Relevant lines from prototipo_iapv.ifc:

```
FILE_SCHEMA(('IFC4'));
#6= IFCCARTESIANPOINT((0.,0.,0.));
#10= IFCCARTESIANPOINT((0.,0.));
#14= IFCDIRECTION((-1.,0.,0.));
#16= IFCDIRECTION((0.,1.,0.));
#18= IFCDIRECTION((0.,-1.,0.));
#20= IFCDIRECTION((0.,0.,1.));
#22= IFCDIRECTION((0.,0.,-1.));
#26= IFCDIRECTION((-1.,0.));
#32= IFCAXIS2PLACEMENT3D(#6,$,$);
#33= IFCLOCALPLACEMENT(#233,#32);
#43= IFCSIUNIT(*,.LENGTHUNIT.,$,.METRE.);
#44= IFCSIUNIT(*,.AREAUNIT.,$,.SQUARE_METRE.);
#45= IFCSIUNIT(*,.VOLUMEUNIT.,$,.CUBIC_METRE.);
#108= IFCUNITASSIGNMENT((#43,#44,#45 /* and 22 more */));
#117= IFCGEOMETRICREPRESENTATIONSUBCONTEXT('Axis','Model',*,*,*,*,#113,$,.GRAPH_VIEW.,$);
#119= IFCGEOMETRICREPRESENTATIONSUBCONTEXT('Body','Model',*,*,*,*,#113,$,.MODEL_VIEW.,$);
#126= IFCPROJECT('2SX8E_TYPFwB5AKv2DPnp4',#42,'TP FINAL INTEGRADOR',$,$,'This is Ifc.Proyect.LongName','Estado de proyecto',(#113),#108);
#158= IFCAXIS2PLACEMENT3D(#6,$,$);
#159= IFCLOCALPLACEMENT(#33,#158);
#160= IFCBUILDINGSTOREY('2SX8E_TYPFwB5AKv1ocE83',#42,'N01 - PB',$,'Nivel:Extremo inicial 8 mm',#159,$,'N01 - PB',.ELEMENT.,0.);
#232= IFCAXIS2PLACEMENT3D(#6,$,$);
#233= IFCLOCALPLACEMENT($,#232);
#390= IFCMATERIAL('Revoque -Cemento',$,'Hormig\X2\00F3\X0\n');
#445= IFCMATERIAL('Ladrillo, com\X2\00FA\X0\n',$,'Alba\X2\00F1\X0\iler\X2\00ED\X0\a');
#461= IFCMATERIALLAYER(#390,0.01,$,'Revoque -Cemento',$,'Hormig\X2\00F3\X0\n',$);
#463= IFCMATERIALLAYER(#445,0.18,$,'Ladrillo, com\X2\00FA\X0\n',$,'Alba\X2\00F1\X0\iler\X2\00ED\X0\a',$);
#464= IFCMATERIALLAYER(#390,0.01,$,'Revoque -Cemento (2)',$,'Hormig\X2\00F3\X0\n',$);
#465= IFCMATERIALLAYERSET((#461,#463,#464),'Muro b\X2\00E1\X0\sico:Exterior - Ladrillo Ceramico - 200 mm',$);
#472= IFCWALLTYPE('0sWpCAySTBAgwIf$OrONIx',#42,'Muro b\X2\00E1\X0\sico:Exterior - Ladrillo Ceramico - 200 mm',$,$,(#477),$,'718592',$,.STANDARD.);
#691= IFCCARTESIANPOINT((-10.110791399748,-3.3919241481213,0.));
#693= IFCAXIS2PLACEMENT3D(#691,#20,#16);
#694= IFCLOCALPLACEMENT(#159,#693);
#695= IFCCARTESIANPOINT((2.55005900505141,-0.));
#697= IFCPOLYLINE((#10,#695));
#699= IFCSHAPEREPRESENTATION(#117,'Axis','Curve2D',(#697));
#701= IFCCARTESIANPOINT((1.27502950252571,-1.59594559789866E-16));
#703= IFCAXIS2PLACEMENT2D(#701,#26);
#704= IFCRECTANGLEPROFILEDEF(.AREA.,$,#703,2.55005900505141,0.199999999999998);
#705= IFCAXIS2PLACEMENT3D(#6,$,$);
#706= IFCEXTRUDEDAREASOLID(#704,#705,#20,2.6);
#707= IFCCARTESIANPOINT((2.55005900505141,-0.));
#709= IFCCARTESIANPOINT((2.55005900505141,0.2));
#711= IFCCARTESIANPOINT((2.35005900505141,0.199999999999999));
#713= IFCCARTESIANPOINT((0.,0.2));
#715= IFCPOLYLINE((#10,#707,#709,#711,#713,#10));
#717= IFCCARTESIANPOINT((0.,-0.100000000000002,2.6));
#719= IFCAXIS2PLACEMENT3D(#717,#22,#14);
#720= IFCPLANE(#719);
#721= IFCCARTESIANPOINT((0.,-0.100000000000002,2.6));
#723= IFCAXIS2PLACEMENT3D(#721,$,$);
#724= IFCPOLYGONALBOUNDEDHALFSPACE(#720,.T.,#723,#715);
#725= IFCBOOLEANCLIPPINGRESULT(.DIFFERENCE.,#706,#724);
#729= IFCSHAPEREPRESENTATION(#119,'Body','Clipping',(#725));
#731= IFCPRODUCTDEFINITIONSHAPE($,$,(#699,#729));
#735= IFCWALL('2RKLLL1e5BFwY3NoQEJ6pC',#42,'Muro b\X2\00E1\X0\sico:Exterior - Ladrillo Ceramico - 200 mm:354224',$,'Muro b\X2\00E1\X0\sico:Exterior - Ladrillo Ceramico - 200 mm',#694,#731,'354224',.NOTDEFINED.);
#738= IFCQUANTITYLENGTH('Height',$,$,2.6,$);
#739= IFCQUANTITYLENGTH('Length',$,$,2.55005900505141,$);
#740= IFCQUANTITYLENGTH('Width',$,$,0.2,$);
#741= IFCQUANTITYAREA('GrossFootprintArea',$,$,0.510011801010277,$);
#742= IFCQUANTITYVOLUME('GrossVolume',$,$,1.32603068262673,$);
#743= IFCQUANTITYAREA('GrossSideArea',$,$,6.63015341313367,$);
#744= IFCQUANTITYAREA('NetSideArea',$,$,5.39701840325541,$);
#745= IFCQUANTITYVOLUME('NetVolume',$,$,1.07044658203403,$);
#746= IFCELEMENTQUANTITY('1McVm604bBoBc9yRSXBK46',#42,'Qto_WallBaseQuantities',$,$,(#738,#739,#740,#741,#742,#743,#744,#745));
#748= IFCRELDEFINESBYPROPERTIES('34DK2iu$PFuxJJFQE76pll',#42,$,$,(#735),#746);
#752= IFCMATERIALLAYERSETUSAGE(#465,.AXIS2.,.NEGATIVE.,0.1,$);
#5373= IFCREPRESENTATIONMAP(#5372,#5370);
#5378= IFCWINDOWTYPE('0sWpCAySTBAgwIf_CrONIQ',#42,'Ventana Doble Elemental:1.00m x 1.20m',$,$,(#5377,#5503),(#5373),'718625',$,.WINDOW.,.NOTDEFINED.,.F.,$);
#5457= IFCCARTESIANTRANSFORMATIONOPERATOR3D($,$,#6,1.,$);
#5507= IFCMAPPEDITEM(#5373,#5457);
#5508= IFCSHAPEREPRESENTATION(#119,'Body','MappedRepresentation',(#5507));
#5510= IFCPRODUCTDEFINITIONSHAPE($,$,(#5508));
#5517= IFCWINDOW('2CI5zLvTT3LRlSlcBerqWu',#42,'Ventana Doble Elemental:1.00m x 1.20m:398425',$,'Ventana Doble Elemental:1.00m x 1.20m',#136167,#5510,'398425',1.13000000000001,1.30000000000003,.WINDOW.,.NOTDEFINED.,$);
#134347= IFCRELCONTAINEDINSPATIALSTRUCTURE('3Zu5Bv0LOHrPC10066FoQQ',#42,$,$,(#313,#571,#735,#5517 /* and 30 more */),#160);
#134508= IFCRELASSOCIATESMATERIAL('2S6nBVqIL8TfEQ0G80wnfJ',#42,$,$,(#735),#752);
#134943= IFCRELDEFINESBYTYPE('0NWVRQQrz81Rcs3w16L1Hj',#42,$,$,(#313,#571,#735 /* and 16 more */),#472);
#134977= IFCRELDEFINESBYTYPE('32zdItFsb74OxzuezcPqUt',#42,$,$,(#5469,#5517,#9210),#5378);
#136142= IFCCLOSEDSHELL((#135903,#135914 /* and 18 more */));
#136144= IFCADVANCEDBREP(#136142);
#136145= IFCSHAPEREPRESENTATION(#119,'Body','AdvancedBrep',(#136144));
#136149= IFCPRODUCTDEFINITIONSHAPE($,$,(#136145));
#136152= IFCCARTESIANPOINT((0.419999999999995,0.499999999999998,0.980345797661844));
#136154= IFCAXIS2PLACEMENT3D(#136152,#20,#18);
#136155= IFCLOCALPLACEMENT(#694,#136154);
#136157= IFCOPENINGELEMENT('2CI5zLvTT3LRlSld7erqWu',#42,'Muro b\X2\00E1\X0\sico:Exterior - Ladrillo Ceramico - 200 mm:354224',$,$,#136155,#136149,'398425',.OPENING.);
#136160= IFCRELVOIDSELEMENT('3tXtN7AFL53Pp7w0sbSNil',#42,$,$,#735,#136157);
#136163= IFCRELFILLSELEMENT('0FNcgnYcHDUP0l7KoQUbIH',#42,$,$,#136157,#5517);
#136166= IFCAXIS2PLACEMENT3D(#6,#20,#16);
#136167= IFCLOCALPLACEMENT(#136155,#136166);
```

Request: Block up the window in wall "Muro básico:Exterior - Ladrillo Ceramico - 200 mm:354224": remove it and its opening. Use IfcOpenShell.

```python
import ifcopenshell
import ifcopenshell.api.feature
import ifcopenshell.api.pset
import ifcopenshell.api.root
import ifcopenshell.geom
import ifcopenshell.util.element
import ifcopenshell.util.shape
import ifcopenshell.util.unit

model = ifcopenshell.open("prototipo_iapv.ifc")
area_scale = ifcopenshell.util.unit.calculate_unit_scale(model, "AREAUNIT")
volume_scale = ifcopenshell.util.unit.calculate_unit_scale(model, "VOLUMEUNIT")
settings = ifcopenshell.geom.settings()


def volume(element):
    """Net volume in cubic metres, openings subtracted."""
    shape = ifcopenshell.geom.create_shape(settings, element)
    return ifcopenshell.util.shape.get_volume(shape.geometry)


window = model.by_id(5517)
opening = window.FillsVoids[0].RelatingOpeningElement
wall = opening.VoidsElements[0].RelatingBuildingElement
before = volume(wall)

ifcopenshell.api.root.remove_product(model, product=window)
ifcopenshell.api.feature.remove_feature(model, feature=opening)

after = volume(wall)
thickness = 0.2  # wall thickness in metres

# Update the wall's stored quantities.
qto = model.by_id(ifcopenshell.util.element.get_pset(wall, "Qto_WallBaseQuantities", should_inherit=False)["id"])
ifcopenshell.api.pset.edit_qto(model, qto=qto, properties={
    "NetSideArea": after / thickness / area_scale,
    "NetVolume": after / volume_scale,
})

print(f"wall volume {before:.3f} -> {after:.3f} m3")

model.write("prototipo_iapv-out.ifc")
```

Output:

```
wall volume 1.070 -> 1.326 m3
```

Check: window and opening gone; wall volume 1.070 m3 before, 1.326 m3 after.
